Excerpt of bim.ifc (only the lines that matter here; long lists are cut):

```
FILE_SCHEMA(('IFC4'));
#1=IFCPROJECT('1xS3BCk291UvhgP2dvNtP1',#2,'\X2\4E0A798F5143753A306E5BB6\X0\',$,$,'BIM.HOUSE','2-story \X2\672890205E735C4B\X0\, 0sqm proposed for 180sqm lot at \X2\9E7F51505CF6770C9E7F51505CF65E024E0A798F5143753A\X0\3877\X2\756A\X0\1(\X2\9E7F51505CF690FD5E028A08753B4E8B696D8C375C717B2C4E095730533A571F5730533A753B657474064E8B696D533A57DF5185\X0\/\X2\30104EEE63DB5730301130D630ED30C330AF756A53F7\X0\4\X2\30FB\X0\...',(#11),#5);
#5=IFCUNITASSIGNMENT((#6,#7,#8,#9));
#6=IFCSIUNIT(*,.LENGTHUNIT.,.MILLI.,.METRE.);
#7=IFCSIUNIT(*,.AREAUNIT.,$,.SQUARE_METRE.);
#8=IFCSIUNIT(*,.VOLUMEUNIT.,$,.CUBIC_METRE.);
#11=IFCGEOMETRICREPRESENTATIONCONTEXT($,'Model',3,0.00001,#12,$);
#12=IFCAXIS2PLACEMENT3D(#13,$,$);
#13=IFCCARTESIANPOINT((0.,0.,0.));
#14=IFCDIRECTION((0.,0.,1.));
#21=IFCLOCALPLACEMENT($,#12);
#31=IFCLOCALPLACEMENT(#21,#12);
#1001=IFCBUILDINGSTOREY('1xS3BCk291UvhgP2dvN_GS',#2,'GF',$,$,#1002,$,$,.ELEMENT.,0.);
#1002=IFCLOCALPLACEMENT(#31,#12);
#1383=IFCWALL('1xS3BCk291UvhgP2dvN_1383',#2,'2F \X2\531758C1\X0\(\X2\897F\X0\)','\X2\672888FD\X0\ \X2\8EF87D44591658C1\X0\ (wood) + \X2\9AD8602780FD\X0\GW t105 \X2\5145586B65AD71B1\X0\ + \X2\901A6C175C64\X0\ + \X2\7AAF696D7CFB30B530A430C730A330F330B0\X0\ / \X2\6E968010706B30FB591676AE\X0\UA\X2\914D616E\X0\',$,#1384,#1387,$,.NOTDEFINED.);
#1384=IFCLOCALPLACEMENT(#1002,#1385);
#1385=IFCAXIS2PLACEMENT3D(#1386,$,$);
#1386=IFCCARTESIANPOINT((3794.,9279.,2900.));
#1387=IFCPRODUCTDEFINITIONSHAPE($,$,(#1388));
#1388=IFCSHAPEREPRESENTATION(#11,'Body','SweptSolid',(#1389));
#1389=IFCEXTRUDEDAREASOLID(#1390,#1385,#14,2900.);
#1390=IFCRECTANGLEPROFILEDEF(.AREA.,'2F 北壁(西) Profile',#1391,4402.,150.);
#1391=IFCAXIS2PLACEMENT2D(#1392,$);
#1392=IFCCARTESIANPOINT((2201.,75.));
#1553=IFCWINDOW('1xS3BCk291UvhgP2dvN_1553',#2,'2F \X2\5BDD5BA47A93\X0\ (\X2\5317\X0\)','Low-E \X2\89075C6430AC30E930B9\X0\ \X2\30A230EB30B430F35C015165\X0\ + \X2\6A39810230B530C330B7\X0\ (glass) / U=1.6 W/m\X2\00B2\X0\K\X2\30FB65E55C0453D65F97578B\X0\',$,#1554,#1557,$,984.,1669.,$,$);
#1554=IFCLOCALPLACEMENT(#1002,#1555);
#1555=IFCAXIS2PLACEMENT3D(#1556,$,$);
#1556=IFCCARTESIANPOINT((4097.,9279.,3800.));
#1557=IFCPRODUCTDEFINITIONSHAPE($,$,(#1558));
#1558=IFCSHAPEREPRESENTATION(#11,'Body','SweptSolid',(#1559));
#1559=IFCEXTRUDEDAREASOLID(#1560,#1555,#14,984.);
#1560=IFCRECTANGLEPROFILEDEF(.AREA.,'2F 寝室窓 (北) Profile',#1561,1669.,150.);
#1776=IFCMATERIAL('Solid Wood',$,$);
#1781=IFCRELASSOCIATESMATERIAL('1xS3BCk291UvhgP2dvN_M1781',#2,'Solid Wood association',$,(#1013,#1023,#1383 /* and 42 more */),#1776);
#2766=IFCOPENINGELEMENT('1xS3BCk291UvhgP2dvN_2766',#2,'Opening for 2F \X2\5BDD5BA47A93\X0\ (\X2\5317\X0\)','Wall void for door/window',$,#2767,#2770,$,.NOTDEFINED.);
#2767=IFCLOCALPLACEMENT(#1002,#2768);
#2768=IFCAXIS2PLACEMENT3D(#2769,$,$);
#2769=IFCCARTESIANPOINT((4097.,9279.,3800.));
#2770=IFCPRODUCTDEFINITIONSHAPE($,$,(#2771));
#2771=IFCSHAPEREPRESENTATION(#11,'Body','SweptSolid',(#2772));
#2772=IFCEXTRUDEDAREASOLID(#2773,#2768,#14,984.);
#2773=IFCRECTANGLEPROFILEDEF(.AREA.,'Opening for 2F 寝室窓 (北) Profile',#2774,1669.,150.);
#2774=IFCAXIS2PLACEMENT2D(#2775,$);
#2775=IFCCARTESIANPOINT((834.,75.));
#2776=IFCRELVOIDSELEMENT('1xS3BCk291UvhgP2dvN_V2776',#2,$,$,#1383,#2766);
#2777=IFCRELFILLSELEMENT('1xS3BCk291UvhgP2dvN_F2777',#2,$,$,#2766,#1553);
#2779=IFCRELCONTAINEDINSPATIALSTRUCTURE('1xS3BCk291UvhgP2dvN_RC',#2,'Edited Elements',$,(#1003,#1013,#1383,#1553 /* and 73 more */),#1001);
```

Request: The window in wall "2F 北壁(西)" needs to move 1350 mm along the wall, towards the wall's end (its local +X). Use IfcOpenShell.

```python
import ifcopenshell
import ifcopenshell.api.geometry
import ifcopenshell.util.placement

model = ifcopenshell.open("bim.ifc")

window = model.by_guid("1xS3BCk291UvhgP2dvN_1553")
opening = window.FillsVoids[0].RelatingOpeningElement
wall = opening.VoidsElements[0].RelatingBuildingElement

wall_matrix = ifcopenshell.util.placement.get_local_placement(wall.ObjectPlacement)
shift = wall_matrix[:3, 0] * 1350.0
before = ifcopenshell.util.placement.get_local_placement(window.ObjectPlacement)[:3, 3].copy()

# The window is not placed relative to its opening, so move both.
for product in (opening, window):
    matrix = ifcopenshell.util.placement.get_local_placement(product.ObjectPlacement)
    matrix[:3, 3] += shift
    ifcopenshell.api.geometry.edit_object_placement(model, product=product, matrix=matrix, is_si=False)

after = ifcopenshell.util.placement.get_local_placement(window.ObjectPlacement)[:3, 3]
print("window moved by", (after - before).round(3) + 0.0)

model.write("bim_rev.ifc")
```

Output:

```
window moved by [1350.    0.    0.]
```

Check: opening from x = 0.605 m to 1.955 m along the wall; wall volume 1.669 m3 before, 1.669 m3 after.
